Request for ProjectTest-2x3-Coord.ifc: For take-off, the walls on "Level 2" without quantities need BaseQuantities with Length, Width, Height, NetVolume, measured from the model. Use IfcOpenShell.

First a look at what the model holds.

```python
import ifcopenshell
import ifcopenshell.util.element
import ifcopenshell.util.unit

model = ifcopenshell.open("ProjectTest-2x3-Coord.ifc")
print(model.schema)
for unit_type in ("LENGTHUNIT", "AREAUNIT", "VOLUMEUNIT"):
    print(unit_type, ifcopenshell.util.unit.calculate_unit_scale(model, unit_type))
storey = next(s for s in model.by_type("IfcBuildingStorey") if s.Name == "Level 2")
walls = [e for e in ifcopenshell.util.element.get_decomposition(storey) if e.is_a("IfcWall")]
for e in sorted(walls, key=lambda e: e.id()):
    print(e.id(), e.is_a(), e.Name, list(ifcopenshell.util.element.get_psets(e, qtos_only=True)), sep=" | ")
```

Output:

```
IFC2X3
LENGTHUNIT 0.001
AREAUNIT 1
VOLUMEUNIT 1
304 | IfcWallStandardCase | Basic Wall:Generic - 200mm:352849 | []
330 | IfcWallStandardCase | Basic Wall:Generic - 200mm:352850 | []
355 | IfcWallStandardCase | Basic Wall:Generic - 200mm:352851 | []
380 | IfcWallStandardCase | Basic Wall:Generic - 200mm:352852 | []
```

```python
import ifcopenshell
import ifcopenshell.api.pset
import ifcopenshell.geom
import ifcopenshell.util.element
import ifcopenshell.util.shape
import ifcopenshell.util.unit

model = ifcopenshell.open("ProjectTest-2x3-Coord.ifc")
unit_scale = ifcopenshell.util.unit.calculate_unit_scale(model)
volume_scale = ifcopenshell.util.unit.calculate_unit_scale(model, "VOLUMEUNIT")
settings = ifcopenshell.geom.settings()

storey = next(s for s in model.by_type("IfcBuildingStorey") if s.Name == "Level 2")
walls = [e for e in ifcopenshell.util.element.get_decomposition(storey) if e.is_a("IfcWall")]

for e in sorted(walls, key=lambda e: e.id()):
    if ifcopenshell.util.element.get_psets(e, qtos_only=True, should_inherit=False):
        continue
    # Geometry comes back in metres, in the element's own axes.
    shape = ifcopenshell.geom.create_shape(settings, e)
    values = {
        "Length": ifcopenshell.util.shape.get_x(shape.geometry) / unit_scale,
        "Width": ifcopenshell.util.shape.get_y(shape.geometry) / unit_scale,
        "Height": ifcopenshell.util.shape.get_z(shape.geometry) / unit_scale,
        "NetVolume": ifcopenshell.util.shape.get_volume(shape.geometry) / volume_scale,
    }
    qto = ifcopenshell.api.pset.add_qto(model, product=e, name="BaseQuantities")
    ifcopenshell.api.pset.edit_qto(model, qto=qto, properties=values)
    print(e.id(), {k: round(v, 3) for k, v in values.items()})

model.write("ProjectTest-2x3-Coord_rev.ifc")
```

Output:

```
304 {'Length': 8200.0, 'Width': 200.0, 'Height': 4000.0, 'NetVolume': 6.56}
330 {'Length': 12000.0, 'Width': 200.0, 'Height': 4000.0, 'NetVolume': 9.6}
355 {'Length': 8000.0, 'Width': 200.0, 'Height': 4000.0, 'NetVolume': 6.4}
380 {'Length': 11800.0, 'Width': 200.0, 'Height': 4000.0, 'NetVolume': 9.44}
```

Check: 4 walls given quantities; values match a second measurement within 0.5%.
